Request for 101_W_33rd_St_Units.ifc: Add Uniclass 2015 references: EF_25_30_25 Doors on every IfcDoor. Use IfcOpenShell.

First a look at what the model holds.

```python
import ifcopenshell

model = ifcopenshell.open("101_W_33rd_St_Units.ifc")
print(model.schema)
print("classifications:", [c.Name for c in model.by_type("IfcClassification")])
for ifc_class in ("IfcDoor", "IfcRoof", "IfcStair", "IfcWall", "IfcWindow"):
    print(ifc_class, len(model.by_type(ifc_class)))
```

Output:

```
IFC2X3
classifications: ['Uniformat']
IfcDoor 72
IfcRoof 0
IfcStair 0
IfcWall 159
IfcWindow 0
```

```python
import ifcopenshell
import ifcopenshell.api.classification

model = ifcopenshell.open("101_W_33rd_St_Units.ifc")

# IFC2X3 requires Source and Edition and has no link from the project to the system.
system = model.create_entity("IfcClassification", Source="NBS", Edition="2015", Name="Uniclass 2015")

codes = {
    "IfcDoor": ("EF_25_30_25", "Doors"),
}
for ifc_class, (code, name) in codes.items():
    products = model.by_type(ifc_class)
    ifcopenshell.api.classification.add_reference(
        model, products=products, classification=system, identification=code, name=name
    )
    print(code, len(products))

model.write("101_W_33rd_St_Units_v2.ifc")
```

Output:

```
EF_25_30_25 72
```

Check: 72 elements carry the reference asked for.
